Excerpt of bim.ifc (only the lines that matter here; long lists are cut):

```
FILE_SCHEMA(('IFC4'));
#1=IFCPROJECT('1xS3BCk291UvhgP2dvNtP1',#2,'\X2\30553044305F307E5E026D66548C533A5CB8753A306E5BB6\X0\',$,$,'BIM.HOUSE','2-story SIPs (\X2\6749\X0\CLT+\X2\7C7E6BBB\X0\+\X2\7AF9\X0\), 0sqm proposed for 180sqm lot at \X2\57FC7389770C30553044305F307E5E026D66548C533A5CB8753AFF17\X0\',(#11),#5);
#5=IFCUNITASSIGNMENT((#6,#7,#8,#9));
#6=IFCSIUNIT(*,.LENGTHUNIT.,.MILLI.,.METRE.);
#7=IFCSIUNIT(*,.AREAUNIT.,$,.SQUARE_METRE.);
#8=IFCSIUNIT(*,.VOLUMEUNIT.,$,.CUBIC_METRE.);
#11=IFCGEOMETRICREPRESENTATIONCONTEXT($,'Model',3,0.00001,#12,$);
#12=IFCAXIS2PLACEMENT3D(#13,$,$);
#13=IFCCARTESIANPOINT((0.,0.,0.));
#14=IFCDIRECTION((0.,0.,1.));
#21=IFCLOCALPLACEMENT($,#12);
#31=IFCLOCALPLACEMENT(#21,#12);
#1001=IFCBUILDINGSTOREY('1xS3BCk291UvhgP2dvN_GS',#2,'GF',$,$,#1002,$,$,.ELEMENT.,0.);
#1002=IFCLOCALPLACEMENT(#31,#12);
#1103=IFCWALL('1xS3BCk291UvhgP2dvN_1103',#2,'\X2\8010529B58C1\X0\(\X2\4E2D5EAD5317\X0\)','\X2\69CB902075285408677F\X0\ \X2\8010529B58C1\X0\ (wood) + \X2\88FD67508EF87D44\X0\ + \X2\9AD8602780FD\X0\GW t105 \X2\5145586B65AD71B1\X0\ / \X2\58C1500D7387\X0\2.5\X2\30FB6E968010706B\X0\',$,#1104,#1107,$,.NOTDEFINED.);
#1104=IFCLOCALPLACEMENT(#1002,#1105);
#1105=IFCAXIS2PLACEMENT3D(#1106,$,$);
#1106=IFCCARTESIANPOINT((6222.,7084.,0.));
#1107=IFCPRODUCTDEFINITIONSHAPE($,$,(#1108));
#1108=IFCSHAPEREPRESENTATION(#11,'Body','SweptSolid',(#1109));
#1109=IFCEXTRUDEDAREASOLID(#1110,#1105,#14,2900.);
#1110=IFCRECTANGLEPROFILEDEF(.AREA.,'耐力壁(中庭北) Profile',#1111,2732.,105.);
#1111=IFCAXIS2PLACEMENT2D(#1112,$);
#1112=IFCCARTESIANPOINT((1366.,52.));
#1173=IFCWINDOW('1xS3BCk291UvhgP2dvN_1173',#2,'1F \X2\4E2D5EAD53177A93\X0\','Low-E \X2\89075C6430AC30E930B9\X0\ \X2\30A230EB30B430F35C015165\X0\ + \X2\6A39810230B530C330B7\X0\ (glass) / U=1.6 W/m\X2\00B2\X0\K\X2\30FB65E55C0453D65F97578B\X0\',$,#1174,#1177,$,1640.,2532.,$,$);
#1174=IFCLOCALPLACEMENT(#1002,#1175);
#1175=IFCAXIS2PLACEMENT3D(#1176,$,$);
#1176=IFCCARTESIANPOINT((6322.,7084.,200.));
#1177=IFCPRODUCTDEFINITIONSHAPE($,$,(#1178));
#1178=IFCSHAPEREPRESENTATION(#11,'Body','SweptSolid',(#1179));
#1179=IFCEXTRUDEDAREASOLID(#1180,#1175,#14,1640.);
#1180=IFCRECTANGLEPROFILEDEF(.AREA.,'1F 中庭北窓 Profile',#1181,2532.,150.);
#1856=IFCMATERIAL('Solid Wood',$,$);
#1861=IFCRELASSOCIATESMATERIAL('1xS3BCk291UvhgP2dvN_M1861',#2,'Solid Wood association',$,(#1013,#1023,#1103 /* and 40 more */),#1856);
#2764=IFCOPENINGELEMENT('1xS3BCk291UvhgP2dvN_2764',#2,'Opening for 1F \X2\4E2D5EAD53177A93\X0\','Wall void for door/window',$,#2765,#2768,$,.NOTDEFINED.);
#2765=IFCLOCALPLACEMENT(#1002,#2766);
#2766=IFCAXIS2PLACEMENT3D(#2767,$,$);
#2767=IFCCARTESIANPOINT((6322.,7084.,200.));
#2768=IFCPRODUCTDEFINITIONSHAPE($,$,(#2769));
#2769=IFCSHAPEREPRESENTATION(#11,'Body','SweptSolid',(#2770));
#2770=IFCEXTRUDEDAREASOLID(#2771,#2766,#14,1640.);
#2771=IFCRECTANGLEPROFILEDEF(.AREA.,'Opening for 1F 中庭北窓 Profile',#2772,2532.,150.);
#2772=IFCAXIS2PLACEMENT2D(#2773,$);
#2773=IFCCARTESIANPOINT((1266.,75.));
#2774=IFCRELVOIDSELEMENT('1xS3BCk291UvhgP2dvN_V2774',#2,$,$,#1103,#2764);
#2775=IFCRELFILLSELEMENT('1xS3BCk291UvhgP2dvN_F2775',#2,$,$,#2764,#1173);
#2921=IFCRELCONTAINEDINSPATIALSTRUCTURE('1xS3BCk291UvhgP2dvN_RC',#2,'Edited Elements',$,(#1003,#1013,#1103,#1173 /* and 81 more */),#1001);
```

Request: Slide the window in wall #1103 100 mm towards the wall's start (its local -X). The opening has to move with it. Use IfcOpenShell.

```python
import ifcopenshell
import ifcopenshell.api.geometry
import ifcopenshell.util.placement
import ifcopenshell.util.unit

model = ifcopenshell.open("bim.ifc")
unit_scale = ifcopenshell.util.unit.calculate_unit_scale(model)

window = model.by_guid("1xS3BCk291UvhgP2dvN_1173")
opening = window.FillsVoids[0].RelatingOpeningElement
wall = opening.VoidsElements[0].RelatingBuildingElement

wall_matrix = ifcopenshell.util.placement.get_local_placement(wall.ObjectPlacement)
shift = wall_matrix[:3, 0] * -0.1 / unit_scale
before = ifcopenshell.util.placement.get_local_placement(window.ObjectPlacement)[:3, 3].copy()

# The window is not placed relative to its opening, so move both.
for product in (opening, window):
    matrix = ifcopenshell.util.placement.get_local_placement(product.ObjectPlacement)
    matrix[:3, 3] += shift
    ifcopenshell.api.geometry.edit_object_placement(model, product=product, matrix=matrix, is_si=False)

after = ifcopenshell.util.placement.get_local_placement(window.ObjectPlacement)[:3, 3]
print("window moved by", (after - before).round(3) + 0.0)

model.write("bim_v2.ifc")
```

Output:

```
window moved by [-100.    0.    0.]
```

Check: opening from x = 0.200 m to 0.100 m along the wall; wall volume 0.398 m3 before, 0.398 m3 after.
